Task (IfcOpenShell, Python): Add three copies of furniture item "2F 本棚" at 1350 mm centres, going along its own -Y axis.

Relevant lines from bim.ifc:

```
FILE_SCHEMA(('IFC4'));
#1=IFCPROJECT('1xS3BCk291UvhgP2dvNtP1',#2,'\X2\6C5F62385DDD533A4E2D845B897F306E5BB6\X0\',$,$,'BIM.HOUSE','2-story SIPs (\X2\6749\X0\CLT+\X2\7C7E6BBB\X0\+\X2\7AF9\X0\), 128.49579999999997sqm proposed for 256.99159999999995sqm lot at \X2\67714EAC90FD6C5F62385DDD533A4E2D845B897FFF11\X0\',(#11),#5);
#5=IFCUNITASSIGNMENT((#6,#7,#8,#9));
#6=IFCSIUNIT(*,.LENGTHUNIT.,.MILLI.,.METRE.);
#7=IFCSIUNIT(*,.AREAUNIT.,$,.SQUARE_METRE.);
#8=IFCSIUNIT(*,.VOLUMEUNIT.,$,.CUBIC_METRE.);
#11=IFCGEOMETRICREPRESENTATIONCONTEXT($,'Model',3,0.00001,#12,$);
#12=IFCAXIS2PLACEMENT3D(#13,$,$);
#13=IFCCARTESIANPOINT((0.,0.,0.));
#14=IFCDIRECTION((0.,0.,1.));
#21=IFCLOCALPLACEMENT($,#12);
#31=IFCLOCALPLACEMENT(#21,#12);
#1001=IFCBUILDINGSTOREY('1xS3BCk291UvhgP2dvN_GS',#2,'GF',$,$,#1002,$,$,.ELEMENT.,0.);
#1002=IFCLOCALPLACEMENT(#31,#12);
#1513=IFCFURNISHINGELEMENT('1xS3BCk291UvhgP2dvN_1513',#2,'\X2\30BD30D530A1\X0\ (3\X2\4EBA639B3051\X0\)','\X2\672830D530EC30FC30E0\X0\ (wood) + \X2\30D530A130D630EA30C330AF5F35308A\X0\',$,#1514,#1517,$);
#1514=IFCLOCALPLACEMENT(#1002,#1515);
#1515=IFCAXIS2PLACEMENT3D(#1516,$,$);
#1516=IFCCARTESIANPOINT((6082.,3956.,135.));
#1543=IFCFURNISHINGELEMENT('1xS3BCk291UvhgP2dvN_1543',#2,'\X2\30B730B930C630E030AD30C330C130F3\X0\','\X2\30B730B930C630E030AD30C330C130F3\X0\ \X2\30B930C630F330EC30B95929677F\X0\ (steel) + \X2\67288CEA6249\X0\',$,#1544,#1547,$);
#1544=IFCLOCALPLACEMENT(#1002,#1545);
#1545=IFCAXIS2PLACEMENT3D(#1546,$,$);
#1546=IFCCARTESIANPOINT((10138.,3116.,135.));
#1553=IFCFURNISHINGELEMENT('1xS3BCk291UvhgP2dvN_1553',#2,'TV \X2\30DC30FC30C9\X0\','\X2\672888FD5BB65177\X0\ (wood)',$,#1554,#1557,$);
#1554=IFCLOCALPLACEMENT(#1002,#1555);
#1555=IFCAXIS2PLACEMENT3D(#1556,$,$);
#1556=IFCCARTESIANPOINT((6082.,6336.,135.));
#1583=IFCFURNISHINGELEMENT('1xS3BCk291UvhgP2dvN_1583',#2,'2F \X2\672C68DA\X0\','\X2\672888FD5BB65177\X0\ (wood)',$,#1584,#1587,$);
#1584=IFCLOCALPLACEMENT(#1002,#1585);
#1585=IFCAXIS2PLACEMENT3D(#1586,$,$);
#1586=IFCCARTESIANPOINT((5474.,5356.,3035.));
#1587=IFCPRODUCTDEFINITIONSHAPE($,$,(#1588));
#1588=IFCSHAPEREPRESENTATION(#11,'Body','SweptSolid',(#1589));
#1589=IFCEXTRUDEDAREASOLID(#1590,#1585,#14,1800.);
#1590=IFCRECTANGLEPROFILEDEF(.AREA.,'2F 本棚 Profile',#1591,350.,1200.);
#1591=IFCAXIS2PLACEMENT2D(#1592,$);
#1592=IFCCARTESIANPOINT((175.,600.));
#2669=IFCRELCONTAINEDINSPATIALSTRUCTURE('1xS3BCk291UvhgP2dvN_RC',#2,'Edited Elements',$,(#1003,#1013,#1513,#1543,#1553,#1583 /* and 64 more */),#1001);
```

```python
import ifcopenshell
import ifcopenshell.api.geometry
import ifcopenshell.api.root
import ifcopenshell.util.element
import ifcopenshell.util.placement

model = ifcopenshell.open("bim.ifc")


def reuse_history(source, copy):
    """copy_class also copies each property set's owner history, people and application; keep the originals."""
    for rel in copy.IsDefinedBy:
        if rel.is_a("IfcRelDefinesByProperties") and (history := rel.RelatingPropertyDefinition.OwnerHistory):
            rel.RelatingPropertyDefinition.OwnerHistory = source.OwnerHistory
            ifcopenshell.util.element.remove_deep2(model, history)


source = model.by_guid("1xS3BCk291UvhgP2dvN_1583")
base = ifcopenshell.util.placement.get_local_placement(source.ObjectPlacement)
step = -base[:3, 1] * 1350.0

for i in range(1, 4):
    copy = ifcopenshell.api.root.copy_class(model, product=source)
    copy.Representation = ifcopenshell.util.element.copy_deep(
        model, source.Representation, exclude=["IfcGeometricRepresentationContext", "IfcRepresentationMap"]
    )
    reuse_history(source, copy)
    matrix = base.copy()
    matrix[:3, 3] += i * step
    print("added at", matrix[:3, 3].round(3) + 0.0)
    ifcopenshell.api.geometry.edit_object_placement(model, product=copy, matrix=matrix, is_si=False)

model.write("bim_updated.ifc")
```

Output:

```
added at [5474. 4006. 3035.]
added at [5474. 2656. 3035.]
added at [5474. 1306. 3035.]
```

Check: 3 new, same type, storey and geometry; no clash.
